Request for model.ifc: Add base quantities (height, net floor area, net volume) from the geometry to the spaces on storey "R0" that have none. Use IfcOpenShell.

First a look at what the model holds.

```python
import ifcopenshell
import ifcopenshell.util.element
import ifcopenshell.util.unit

model = ifcopenshell.open("model.ifc")
print(model.schema)
for unit_type in ("LENGTHUNIT", "AREAUNIT", "VOLUMEUNIT"):
    print(unit_type, ifcopenshell.util.unit.calculate_unit_scale(model, unit_type))
storey = next(s for s in model.by_type("IfcBuildingStorey") if s.Name == "R0")
spaces = [e for e in ifcopenshell.util.element.get_decomposition(storey) if e.is_a("IfcSpace")]
for e in sorted(spaces, key=lambda e: e.id()):
    print(e.id(), e.is_a(), e.Name, list(ifcopenshell.util.element.get_psets(e, qtos_only=True)), sep=" | ")
```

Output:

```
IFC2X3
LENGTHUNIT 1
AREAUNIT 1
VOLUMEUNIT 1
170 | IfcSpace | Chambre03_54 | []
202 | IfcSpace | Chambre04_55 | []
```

```python
import ifcopenshell
import ifcopenshell.api.pset
import ifcopenshell.geom
import ifcopenshell.util.element
import ifcopenshell.util.shape
import ifcopenshell.util.unit

model = ifcopenshell.open("model.ifc")
unit_scale = ifcopenshell.util.unit.calculate_unit_scale(model)
area_scale = ifcopenshell.util.unit.calculate_unit_scale(model, "AREAUNIT")
volume_scale = ifcopenshell.util.unit.calculate_unit_scale(model, "VOLUMEUNIT")
settings = ifcopenshell.geom.settings()

storey = next(s for s in model.by_type("IfcBuildingStorey") if s.Name == "R0")
spaces = [e for e in ifcopenshell.util.element.get_decomposition(storey) if e.is_a("IfcSpace")]

for e in sorted(spaces, key=lambda e: e.id()):
    if ifcopenshell.util.element.get_psets(e, qtos_only=True, should_inherit=False):
        continue
    # Geometry comes back in metres, in the element's own axes.
    shape = ifcopenshell.geom.create_shape(settings, e)
    values = {
        "Height": ifcopenshell.util.shape.get_z(shape.geometry) / unit_scale,
        "NetFloorArea": ifcopenshell.util.shape.get_footprint_area(shape.geometry) / area_scale,
        "NetVolume": ifcopenshell.util.shape.get_volume(shape.geometry) / volume_scale,
    }
    qto = ifcopenshell.api.pset.add_qto(model, product=e, name="BaseQuantities")
    ifcopenshell.api.pset.edit_qto(model, qto=qto, properties=values)
    print(e.id(), {k: round(v, 3) for k, v in values.items()})

model.write("model_rev.ifc")
```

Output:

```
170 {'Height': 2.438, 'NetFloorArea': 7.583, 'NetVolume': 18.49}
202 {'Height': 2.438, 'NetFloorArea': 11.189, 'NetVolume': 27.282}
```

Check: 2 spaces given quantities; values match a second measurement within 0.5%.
